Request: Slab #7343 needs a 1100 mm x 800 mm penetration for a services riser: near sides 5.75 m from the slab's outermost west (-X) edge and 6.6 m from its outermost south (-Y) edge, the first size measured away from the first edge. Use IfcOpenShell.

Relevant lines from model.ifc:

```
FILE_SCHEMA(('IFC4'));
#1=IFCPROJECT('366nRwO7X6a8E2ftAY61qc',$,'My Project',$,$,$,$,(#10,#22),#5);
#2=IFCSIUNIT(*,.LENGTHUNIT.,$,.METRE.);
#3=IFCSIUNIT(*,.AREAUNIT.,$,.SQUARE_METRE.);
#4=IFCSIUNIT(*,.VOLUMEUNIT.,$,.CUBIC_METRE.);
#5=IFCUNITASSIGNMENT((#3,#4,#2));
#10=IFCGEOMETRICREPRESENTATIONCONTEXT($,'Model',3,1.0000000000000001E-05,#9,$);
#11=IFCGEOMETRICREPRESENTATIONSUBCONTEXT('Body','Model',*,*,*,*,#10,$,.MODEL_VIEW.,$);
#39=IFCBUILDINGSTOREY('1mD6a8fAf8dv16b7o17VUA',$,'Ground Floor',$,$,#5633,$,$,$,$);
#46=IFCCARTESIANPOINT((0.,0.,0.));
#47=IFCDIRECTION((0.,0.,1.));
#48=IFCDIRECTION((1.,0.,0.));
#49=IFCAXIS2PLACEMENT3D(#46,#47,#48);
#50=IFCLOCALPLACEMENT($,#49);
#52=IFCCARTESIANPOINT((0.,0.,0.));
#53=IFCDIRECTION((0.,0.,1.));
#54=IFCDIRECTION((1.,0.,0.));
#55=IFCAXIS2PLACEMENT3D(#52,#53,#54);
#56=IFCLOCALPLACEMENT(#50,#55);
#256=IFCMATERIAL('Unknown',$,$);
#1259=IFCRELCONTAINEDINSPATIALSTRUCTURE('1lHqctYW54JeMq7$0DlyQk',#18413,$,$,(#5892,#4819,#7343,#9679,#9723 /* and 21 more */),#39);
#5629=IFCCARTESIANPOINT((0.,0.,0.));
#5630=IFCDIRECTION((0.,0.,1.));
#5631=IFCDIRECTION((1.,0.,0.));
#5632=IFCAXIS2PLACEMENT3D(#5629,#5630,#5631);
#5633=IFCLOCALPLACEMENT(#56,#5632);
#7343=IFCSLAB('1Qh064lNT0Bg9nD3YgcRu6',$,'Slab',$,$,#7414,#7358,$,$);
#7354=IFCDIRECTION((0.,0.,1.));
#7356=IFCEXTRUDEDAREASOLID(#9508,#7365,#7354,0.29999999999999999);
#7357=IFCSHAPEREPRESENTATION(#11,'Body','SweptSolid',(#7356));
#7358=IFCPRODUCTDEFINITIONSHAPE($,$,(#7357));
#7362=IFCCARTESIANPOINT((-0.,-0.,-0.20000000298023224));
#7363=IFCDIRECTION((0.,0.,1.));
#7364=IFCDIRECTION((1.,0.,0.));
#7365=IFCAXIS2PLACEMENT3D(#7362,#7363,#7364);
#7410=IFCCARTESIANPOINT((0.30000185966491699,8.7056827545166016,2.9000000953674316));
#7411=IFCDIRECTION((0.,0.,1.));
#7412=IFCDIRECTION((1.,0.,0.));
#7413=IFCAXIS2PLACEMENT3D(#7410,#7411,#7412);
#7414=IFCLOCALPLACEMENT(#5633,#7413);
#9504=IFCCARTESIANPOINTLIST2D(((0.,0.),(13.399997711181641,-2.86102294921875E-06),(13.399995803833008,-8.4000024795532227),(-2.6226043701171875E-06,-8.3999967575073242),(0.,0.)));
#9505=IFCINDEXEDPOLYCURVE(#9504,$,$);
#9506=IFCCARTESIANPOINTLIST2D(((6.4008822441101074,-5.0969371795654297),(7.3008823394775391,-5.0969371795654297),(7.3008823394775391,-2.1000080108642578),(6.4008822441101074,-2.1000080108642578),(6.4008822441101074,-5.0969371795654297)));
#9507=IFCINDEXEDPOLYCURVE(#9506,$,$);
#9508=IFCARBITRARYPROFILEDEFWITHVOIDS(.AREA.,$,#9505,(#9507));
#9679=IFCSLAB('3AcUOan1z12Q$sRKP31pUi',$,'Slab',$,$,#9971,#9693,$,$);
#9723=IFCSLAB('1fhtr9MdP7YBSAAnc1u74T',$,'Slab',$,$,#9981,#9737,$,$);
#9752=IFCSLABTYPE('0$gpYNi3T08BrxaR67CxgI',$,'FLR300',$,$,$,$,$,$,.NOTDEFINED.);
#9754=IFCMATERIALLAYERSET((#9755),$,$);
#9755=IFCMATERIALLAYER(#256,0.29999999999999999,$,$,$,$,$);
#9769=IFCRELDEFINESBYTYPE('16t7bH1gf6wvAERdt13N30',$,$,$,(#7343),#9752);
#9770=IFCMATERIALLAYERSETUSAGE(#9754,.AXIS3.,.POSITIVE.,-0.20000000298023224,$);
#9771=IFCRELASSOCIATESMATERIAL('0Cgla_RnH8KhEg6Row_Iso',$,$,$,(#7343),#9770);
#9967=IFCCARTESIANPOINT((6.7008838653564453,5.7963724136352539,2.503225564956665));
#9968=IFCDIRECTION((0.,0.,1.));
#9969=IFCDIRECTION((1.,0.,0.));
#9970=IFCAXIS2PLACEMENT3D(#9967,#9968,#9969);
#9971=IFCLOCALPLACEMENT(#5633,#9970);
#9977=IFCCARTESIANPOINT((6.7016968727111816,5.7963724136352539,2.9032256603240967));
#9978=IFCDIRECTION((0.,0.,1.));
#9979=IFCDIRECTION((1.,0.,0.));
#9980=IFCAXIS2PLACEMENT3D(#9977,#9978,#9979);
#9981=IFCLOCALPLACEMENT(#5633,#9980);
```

```python
import numpy as np
import ifcopenshell
import ifcopenshell.api.feature
import ifcopenshell.api.geometry
import ifcopenshell.api.root
import ifcopenshell.geom
import ifcopenshell.util.placement
import ifcopenshell.util.representation
import ifcopenshell.util.shape
import ifcopenshell.util.unit

model = ifcopenshell.open("model.ifc")
unit_scale = ifcopenshell.util.unit.calculate_unit_scale(model)
settings = ifcopenshell.geom.settings()


def volume(element):
    """Net volume in cubic metres, openings subtracted."""
    shape = ifcopenshell.geom.create_shape(settings, element)
    return ifcopenshell.util.shape.get_volume(shape.geometry)


slab = model.by_guid("1Qh064lNT0Bg9nD3YgcRu6")
before = volume(slab)

# Extent in the slab's own axes, in metres. The edges named are its -X and -Y sides.
slab_shape = ifcopenshell.geom.create_shape(settings, slab)
vertices = ifcopenshell.util.shape.get_vertices(slab_shape.geometry)
x_min, y_min, bottom = vertices.min(axis=0)
top = vertices[:, 2].max()

opening = ifcopenshell.api.root.create_entity(model, ifc_class="IfcOpeningElement", name="Services riser opening", predefined_type="OPENING")
context = ifcopenshell.util.representation.get_context(model, "Model", "Body", "MODEL_VIEW")
width, depth = 1.1, 0.8
outline = [(0.0, 0.0), (width, 0.0), (width, depth), (0.0, depth), (0.0, 0.0)]
# Overshoot both faces by 50 mm so the cut is clean.
shape = ifcopenshell.api.geometry.add_slab_representation(
    model, context=context, depth=top - bottom + 0.1, polyline=outline
)
ifcopenshell.api.geometry.assign_representation(model, product=opening, representation=shape)

matrix = ifcopenshell.util.placement.get_local_placement(slab.ObjectPlacement)
matrix[:, 3] = matrix @ np.append(np.array([x_min + 5.75, y_min + 6.6, bottom - 0.05]) / unit_scale, 1.0)
ifcopenshell.api.geometry.edit_object_placement(model, product=opening, matrix=matrix, is_si=False)
ifcopenshell.api.feature.add_feature(model, feature=opening, element=slab)

after = volume(slab)

print(f"slab volume {before:.3f} -> {after:.3f} m3")

model.write("model-out.ifc")
```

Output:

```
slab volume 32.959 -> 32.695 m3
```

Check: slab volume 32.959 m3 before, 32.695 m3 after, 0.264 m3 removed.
